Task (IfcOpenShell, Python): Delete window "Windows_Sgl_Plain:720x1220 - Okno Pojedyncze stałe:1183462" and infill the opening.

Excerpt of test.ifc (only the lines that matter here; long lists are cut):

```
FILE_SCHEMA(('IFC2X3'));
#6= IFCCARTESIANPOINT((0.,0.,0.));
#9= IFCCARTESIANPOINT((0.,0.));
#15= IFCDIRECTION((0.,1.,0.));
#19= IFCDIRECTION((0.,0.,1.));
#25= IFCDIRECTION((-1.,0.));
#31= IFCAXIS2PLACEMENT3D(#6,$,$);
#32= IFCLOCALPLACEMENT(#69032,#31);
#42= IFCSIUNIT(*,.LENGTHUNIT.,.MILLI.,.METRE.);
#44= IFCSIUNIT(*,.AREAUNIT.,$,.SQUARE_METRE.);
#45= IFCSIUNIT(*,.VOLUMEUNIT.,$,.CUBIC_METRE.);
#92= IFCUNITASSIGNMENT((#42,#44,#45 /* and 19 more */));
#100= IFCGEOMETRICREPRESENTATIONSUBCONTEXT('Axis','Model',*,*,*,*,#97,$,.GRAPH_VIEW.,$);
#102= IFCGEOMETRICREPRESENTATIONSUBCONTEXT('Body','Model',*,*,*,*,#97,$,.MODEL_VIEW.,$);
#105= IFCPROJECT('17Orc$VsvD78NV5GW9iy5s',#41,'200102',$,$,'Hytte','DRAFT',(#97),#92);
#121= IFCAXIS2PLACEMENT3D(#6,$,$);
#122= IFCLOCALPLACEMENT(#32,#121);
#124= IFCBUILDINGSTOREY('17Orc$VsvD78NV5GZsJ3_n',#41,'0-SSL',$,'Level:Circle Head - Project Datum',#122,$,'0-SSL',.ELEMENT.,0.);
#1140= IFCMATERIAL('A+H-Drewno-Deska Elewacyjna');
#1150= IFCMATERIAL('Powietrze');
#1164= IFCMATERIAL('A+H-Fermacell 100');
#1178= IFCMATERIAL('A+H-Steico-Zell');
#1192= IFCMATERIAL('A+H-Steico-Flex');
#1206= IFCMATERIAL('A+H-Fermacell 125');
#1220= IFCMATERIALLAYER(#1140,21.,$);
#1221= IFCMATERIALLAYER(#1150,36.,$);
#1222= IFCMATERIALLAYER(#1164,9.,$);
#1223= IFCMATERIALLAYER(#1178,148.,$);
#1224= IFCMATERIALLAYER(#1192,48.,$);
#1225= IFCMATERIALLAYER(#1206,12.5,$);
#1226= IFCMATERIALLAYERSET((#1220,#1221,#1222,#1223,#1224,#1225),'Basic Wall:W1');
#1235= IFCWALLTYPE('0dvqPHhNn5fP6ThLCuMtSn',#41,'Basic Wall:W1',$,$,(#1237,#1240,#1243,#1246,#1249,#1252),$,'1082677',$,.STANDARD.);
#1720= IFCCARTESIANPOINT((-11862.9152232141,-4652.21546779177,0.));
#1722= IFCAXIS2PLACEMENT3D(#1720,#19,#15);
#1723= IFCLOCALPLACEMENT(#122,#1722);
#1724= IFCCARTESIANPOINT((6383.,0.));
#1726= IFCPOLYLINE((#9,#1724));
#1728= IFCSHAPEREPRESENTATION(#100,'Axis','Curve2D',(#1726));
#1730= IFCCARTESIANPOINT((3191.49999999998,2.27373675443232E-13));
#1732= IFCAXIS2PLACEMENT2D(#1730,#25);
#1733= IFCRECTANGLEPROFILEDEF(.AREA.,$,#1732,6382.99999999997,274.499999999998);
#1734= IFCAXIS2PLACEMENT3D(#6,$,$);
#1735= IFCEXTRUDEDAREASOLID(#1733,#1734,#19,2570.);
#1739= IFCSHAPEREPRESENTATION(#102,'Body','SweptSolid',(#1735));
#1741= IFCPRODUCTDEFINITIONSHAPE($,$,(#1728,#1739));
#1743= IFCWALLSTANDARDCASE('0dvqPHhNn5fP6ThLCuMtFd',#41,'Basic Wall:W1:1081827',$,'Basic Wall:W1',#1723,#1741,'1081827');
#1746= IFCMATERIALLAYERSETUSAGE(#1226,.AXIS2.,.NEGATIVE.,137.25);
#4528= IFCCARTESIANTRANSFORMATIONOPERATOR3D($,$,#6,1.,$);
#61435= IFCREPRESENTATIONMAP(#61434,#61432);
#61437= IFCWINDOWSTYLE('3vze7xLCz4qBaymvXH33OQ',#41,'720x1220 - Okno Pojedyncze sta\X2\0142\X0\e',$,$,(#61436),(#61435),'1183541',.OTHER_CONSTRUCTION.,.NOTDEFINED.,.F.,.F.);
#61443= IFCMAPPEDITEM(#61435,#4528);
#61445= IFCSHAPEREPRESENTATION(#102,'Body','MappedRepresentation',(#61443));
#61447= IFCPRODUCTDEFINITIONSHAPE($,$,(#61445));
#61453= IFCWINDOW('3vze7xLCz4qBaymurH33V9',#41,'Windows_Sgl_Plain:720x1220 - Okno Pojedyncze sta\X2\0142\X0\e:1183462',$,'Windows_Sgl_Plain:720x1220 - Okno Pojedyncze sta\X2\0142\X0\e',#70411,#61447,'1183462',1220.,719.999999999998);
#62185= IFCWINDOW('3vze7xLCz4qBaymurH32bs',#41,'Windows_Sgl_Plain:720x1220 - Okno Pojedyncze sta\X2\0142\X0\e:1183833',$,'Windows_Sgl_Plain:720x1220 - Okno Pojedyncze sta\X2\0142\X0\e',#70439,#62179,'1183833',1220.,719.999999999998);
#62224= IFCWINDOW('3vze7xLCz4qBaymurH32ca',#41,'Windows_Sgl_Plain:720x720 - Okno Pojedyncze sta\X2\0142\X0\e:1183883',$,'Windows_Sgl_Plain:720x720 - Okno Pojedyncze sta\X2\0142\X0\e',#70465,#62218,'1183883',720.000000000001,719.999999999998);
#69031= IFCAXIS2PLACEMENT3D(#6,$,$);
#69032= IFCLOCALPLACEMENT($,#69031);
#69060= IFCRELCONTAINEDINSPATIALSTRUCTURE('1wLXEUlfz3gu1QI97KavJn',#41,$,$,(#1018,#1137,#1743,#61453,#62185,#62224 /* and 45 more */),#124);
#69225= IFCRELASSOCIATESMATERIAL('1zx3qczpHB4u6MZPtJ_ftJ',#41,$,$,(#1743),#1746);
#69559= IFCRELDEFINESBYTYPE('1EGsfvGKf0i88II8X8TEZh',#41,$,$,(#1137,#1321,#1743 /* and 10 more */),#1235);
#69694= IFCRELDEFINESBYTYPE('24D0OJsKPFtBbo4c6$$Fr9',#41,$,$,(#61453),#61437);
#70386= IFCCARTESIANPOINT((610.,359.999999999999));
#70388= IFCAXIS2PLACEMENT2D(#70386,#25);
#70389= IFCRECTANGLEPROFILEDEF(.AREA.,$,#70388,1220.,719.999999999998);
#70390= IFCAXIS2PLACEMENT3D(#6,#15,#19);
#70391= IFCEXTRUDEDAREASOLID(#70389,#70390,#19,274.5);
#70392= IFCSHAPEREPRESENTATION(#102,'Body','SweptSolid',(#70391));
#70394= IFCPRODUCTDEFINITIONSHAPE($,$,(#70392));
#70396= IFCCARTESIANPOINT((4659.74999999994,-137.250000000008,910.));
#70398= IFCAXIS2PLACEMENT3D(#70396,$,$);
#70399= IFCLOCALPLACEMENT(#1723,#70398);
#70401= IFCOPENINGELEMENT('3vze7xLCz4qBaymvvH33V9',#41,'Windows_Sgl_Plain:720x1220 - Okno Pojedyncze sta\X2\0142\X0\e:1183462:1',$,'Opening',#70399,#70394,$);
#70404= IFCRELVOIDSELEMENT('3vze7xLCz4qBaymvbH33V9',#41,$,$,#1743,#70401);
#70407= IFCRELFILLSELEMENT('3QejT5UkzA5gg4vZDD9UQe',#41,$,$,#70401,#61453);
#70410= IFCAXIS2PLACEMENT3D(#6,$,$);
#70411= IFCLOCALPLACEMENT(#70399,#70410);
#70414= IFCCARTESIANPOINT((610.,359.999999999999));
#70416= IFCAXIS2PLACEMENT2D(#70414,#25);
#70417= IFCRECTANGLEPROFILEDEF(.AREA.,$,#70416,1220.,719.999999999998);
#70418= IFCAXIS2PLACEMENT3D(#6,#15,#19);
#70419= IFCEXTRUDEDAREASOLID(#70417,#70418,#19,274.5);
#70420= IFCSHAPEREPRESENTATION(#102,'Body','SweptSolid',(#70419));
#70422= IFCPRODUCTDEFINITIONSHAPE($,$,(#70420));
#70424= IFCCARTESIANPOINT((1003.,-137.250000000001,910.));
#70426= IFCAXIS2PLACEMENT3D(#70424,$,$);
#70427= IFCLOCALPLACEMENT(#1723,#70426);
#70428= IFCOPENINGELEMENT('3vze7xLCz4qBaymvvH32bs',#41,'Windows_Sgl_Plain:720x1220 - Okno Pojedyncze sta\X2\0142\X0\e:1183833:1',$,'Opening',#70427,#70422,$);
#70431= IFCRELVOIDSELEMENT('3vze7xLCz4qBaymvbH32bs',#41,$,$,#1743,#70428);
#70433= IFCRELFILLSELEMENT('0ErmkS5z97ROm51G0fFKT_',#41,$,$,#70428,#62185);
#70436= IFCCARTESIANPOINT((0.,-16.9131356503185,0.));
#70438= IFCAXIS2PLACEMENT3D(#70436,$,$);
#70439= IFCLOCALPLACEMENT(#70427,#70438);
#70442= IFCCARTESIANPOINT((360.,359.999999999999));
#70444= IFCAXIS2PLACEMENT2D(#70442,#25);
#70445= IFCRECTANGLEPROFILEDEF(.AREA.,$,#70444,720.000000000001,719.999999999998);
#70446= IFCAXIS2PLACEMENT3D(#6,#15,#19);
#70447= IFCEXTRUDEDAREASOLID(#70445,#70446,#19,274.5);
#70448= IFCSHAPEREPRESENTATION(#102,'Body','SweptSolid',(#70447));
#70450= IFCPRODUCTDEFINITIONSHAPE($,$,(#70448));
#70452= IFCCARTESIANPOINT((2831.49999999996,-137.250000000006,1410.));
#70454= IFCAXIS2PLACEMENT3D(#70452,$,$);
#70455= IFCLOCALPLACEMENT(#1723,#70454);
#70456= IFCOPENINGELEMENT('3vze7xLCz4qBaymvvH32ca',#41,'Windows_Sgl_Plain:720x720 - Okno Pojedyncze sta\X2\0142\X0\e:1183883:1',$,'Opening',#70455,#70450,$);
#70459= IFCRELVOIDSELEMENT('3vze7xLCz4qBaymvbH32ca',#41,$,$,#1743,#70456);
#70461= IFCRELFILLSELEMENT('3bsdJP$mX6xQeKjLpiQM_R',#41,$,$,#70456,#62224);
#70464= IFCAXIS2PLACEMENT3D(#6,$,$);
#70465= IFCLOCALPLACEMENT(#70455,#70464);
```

```python
import ifcopenshell
import ifcopenshell.api.feature
import ifcopenshell.api.root
import ifcopenshell.geom
import ifcopenshell.util.shape

model = ifcopenshell.open("test.ifc")
settings = ifcopenshell.geom.settings()


def volume(element):
    """Net volume in cubic metres, openings subtracted."""
    shape = ifcopenshell.geom.create_shape(settings, element)
    return ifcopenshell.util.shape.get_volume(shape.geometry)


window = model.by_id(61453)
opening = window.FillsVoids[0].RelatingOpeningElement
wall = opening.VoidsElements[0].RelatingBuildingElement
before = volume(wall)

ifcopenshell.api.root.remove_product(model, product=window)
ifcopenshell.api.feature.remove_feature(model, feature=opening)

after = volume(wall)

print(f"wall volume {before:.3f} -> {after:.3f} m3")

model.write("test_edited.ifc")
```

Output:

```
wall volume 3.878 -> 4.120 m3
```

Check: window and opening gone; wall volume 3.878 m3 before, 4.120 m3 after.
